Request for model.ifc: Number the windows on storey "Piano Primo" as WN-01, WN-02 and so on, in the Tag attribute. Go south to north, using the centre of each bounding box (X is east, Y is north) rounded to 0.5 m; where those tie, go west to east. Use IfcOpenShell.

First a look at what the model holds.

```python
import ifcopenshell
import ifcopenshell.util.element
import ifcopenshell.util.placement

model = ifcopenshell.open("model.ifc")
print(model.schema)
storey = next(s for s in model.by_type("IfcBuildingStorey") if s.Name == "Piano Primo")
windows = [e for e in ifcopenshell.util.element.get_decomposition(storey) if e.is_a("IfcWindow")]
for e in sorted(windows, key=lambda e: e.id()):
    origin = ifcopenshell.util.placement.get_local_placement(e.ObjectPlacement)[:3, 3]
    print(e.id(), e.Tag, e.Name, origin.round(2) + 0.0, sep=" | ")
```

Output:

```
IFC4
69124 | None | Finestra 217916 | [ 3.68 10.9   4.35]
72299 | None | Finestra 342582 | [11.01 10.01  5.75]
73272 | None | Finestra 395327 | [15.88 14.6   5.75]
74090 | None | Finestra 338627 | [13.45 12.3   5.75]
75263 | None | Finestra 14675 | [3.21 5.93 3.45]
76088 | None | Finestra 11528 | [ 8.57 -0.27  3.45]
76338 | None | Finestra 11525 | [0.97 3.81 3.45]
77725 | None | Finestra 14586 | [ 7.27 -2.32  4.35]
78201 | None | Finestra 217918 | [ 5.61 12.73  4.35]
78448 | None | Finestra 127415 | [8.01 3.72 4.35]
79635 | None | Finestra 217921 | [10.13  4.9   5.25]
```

```python
import ifcopenshell
import ifcopenshell.geom
import ifcopenshell.util.element
import ifcopenshell.util.shape

model = ifcopenshell.open("model.ifc")
settings = ifcopenshell.geom.settings()
settings.set("use-world-coords", True)


def centre(element):
    shape = ifcopenshell.geom.create_shape(settings, element)
    return ifcopenshell.util.shape.get_bbox_centroid(shape.geometry)


storey = next(s for s in model.by_type("IfcBuildingStorey") if s.Name == "Piano Primo")
windows = [e for e in ifcopenshell.util.element.get_decomposition(storey) if e.is_a("IfcWindow")]

# Insertion points can sit at a corner or the storey origin, so sort by the geometry (in metres).
centres = {e: centre(e) for e in windows}
windows.sort(key=lambda e: (round(centres[e][1] / 0.5), centres[e][0]))

for i, e in enumerate(windows, start=1):
    number = f"WN-{i:02d}"
    e.Tag = number
    print(e.id(), number)

model.write("model_edited.ifc")
```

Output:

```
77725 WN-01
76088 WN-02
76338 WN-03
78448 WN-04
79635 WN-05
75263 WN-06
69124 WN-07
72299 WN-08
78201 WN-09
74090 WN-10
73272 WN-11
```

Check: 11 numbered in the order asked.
